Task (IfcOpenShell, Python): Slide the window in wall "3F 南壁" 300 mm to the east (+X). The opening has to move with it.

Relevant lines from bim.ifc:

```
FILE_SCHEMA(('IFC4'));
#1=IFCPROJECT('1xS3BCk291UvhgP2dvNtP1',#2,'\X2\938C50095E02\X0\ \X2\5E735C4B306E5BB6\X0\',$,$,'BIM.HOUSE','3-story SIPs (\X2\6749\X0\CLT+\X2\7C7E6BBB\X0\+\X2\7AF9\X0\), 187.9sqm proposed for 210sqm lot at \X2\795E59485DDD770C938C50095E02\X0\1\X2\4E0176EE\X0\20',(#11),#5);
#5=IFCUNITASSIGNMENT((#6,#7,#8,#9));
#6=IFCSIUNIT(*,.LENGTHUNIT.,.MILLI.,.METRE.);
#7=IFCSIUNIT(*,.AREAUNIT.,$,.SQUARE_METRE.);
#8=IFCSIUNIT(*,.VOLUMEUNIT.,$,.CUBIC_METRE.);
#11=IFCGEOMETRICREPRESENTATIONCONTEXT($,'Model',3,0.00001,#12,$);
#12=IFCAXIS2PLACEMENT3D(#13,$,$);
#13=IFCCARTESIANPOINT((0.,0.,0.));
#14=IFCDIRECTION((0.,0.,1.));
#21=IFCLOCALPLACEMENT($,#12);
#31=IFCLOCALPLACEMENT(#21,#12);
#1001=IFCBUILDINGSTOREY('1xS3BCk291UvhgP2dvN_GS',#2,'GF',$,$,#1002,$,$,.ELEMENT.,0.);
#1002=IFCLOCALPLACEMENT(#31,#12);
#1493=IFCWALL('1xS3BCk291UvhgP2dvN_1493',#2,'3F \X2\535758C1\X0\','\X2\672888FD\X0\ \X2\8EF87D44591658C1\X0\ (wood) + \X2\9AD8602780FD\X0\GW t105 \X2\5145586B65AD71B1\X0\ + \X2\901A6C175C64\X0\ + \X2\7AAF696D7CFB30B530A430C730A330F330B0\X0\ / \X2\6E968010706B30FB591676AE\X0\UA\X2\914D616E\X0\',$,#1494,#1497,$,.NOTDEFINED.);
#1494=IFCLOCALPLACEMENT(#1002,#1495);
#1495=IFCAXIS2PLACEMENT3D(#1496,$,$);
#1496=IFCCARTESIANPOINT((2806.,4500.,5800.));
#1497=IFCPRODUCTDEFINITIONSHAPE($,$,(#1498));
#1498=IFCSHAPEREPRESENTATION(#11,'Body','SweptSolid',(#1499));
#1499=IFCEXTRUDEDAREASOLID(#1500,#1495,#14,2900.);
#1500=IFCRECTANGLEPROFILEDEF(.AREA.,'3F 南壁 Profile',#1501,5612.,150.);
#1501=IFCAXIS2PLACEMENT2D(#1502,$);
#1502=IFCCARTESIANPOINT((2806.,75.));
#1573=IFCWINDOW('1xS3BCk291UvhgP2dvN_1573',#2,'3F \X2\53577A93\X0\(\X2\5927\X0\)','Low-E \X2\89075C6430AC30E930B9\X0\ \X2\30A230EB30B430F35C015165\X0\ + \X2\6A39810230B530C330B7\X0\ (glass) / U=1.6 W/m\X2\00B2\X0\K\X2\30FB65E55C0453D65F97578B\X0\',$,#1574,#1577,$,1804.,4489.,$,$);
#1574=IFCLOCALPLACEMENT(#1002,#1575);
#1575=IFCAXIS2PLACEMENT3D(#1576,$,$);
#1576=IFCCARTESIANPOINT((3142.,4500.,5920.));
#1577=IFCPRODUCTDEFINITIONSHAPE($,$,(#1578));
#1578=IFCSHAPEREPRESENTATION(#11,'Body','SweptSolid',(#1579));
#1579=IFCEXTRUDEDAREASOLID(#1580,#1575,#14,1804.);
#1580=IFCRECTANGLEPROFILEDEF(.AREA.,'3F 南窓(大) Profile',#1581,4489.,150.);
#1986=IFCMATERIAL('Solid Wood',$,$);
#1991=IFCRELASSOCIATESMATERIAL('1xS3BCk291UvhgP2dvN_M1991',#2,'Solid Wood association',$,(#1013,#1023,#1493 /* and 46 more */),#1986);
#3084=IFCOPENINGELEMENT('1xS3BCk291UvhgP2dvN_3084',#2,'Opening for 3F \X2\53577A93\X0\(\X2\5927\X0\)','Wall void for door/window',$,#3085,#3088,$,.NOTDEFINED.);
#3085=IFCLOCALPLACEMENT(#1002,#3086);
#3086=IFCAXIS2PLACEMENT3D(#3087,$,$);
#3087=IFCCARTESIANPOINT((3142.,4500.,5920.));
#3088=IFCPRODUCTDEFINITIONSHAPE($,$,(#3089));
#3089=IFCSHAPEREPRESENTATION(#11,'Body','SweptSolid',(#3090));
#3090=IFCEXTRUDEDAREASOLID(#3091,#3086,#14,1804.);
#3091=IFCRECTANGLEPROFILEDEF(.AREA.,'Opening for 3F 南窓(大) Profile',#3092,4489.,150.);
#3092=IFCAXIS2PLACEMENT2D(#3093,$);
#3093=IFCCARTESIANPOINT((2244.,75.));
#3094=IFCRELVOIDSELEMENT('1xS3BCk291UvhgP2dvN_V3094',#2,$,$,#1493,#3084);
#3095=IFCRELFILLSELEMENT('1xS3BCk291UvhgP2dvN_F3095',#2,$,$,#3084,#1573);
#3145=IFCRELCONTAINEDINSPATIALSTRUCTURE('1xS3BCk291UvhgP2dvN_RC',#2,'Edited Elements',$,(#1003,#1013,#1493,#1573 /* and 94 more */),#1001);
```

```python
import ifcopenshell
import ifcopenshell.api.geometry
import ifcopenshell.util.placement
import ifcopenshell.util.unit

model = ifcopenshell.open("bim.ifc")
unit_scale = ifcopenshell.util.unit.calculate_unit_scale(model)

window = model.by_id(1573)
opening = window.FillsVoids[0].RelatingOpeningElement
wall = opening.VoidsElements[0].RelatingBuildingElement

wall_matrix = ifcopenshell.util.placement.get_local_placement(wall.ObjectPlacement)
shift = wall_matrix[:3, 0] * 0.3 / unit_scale
before = ifcopenshell.util.placement.get_local_placement(window.ObjectPlacement)[:3, 3].copy()

# The window is not placed relative to its opening, so move both.
for product in (opening, window):
    matrix = ifcopenshell.util.placement.get_local_placement(product.ObjectPlacement)
    matrix[:3, 3] += shift
    ifcopenshell.api.geometry.edit_object_placement(model, product=product, matrix=matrix, is_si=False)

after = ifcopenshell.util.placement.get_local_placement(window.ObjectPlacement)[:3, 3]
print("window moved by", (after - before).round(3) + 0.0)

model.write("bim_updated.ifc")
```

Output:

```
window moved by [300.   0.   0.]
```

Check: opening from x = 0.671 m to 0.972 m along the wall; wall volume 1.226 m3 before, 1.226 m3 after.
